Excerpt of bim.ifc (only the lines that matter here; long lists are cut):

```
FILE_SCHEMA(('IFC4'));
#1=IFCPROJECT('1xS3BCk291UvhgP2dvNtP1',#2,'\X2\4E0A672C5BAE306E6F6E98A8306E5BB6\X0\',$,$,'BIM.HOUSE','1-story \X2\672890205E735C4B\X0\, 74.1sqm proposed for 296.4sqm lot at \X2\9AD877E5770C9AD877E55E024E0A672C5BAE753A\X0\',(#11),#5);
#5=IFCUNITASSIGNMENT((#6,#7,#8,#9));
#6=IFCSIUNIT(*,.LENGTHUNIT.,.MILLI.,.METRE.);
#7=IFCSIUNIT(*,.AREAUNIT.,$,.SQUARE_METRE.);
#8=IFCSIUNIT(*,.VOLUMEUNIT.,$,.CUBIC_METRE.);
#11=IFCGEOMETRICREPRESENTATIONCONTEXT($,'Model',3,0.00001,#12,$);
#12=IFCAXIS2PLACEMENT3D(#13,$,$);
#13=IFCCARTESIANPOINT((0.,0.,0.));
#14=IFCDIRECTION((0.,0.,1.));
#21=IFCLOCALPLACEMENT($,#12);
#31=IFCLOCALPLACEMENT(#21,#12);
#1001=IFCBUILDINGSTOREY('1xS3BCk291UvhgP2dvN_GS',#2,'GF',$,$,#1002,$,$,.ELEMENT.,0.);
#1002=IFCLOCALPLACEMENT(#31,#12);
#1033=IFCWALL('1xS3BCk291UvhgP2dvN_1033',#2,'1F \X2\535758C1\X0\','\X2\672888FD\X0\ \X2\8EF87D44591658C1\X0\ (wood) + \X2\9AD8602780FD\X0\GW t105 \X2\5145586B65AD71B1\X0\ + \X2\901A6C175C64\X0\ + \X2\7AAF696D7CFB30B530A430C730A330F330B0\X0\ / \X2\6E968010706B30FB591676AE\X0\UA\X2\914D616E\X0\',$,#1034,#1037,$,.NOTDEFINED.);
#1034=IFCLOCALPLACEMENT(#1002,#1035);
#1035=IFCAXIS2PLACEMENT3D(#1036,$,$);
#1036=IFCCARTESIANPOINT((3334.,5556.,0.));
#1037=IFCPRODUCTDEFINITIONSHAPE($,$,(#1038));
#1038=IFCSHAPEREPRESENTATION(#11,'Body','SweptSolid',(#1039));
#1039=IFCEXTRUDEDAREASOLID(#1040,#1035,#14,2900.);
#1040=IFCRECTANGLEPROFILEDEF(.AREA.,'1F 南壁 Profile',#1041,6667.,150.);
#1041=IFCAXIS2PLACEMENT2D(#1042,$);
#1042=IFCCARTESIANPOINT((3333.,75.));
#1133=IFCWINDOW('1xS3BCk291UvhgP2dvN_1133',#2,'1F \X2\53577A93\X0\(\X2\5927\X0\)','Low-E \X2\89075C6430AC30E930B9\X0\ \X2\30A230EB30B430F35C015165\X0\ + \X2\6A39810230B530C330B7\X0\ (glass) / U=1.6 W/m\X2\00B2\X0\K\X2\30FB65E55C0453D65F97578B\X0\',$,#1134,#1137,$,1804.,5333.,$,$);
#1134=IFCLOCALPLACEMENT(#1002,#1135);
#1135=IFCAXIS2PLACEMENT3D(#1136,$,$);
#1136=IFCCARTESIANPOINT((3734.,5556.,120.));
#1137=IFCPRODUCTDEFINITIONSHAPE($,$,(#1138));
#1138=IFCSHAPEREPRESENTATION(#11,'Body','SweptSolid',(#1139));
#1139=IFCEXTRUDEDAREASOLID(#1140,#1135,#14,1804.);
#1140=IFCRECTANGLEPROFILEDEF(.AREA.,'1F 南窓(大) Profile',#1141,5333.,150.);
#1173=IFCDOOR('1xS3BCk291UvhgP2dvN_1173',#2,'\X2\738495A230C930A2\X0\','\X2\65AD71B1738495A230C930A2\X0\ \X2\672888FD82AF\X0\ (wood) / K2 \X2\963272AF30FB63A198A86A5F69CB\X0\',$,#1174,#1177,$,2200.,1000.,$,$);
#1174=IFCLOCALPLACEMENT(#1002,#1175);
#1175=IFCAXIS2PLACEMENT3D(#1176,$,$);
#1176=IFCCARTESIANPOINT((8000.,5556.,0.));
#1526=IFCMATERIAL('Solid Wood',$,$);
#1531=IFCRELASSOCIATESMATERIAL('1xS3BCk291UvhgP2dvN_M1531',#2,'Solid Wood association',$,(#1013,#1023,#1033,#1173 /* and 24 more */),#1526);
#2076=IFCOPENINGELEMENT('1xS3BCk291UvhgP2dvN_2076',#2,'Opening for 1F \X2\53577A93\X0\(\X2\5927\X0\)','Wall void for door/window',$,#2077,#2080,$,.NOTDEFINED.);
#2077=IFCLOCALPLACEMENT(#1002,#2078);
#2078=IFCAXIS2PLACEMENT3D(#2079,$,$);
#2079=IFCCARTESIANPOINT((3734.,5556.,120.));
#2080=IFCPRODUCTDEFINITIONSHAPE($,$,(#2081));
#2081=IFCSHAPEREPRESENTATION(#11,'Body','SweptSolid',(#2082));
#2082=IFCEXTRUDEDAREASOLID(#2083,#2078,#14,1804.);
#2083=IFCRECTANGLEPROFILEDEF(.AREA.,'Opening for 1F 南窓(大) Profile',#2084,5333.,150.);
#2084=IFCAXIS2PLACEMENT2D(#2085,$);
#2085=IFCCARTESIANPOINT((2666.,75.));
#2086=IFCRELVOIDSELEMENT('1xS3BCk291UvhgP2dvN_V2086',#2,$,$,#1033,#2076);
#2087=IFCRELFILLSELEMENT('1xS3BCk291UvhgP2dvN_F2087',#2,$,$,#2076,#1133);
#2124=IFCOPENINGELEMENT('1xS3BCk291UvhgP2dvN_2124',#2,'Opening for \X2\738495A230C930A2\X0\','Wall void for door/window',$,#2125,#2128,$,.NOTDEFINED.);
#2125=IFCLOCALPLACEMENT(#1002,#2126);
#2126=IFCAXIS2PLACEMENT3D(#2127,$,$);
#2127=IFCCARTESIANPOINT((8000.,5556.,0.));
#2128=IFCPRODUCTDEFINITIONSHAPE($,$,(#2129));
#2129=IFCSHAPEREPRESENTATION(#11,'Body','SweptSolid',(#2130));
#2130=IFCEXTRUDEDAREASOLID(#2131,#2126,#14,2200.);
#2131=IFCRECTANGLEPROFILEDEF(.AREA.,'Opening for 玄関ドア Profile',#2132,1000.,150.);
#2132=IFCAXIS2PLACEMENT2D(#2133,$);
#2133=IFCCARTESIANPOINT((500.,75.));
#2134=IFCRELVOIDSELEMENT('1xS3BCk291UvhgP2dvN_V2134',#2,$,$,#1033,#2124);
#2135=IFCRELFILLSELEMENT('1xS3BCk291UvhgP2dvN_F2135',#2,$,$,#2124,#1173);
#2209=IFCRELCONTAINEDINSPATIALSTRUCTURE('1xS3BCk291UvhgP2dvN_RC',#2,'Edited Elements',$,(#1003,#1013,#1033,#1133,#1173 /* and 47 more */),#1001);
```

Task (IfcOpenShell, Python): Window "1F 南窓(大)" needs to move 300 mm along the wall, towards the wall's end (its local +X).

```python
import ifcopenshell
import ifcopenshell.api.geometry
import ifcopenshell.util.placement
import ifcopenshell.util.unit

model = ifcopenshell.open("bim.ifc")
unit_scale = ifcopenshell.util.unit.calculate_unit_scale(model)

window = model.by_guid("1xS3BCk291UvhgP2dvN_1133")
opening = window.FillsVoids[0].RelatingOpeningElement
wall = opening.VoidsElements[0].RelatingBuildingElement

wall_matrix = ifcopenshell.util.placement.get_local_placement(wall.ObjectPlacement)
shift = wall_matrix[:3, 0] * 0.3 / unit_scale
before = ifcopenshell.util.placement.get_local_placement(window.ObjectPlacement)[:3, 3].copy()

# The window is not placed relative to its opening, so move both.
for product in (opening, window):
    matrix = ifcopenshell.util.placement.get_local_placement(product.ObjectPlacement)
    matrix[:3, 3] += shift
    ifcopenshell.api.geometry.edit_object_placement(model, product=product, matrix=matrix, is_si=False)

after = ifcopenshell.util.placement.get_local_placement(window.ObjectPlacement)[:3, 3]
print("window moved by", (after - before).round(3) + 0.0)

model.write("bim_rev.ifc")
```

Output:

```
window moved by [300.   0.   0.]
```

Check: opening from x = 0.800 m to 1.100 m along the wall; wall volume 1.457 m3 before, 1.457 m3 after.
